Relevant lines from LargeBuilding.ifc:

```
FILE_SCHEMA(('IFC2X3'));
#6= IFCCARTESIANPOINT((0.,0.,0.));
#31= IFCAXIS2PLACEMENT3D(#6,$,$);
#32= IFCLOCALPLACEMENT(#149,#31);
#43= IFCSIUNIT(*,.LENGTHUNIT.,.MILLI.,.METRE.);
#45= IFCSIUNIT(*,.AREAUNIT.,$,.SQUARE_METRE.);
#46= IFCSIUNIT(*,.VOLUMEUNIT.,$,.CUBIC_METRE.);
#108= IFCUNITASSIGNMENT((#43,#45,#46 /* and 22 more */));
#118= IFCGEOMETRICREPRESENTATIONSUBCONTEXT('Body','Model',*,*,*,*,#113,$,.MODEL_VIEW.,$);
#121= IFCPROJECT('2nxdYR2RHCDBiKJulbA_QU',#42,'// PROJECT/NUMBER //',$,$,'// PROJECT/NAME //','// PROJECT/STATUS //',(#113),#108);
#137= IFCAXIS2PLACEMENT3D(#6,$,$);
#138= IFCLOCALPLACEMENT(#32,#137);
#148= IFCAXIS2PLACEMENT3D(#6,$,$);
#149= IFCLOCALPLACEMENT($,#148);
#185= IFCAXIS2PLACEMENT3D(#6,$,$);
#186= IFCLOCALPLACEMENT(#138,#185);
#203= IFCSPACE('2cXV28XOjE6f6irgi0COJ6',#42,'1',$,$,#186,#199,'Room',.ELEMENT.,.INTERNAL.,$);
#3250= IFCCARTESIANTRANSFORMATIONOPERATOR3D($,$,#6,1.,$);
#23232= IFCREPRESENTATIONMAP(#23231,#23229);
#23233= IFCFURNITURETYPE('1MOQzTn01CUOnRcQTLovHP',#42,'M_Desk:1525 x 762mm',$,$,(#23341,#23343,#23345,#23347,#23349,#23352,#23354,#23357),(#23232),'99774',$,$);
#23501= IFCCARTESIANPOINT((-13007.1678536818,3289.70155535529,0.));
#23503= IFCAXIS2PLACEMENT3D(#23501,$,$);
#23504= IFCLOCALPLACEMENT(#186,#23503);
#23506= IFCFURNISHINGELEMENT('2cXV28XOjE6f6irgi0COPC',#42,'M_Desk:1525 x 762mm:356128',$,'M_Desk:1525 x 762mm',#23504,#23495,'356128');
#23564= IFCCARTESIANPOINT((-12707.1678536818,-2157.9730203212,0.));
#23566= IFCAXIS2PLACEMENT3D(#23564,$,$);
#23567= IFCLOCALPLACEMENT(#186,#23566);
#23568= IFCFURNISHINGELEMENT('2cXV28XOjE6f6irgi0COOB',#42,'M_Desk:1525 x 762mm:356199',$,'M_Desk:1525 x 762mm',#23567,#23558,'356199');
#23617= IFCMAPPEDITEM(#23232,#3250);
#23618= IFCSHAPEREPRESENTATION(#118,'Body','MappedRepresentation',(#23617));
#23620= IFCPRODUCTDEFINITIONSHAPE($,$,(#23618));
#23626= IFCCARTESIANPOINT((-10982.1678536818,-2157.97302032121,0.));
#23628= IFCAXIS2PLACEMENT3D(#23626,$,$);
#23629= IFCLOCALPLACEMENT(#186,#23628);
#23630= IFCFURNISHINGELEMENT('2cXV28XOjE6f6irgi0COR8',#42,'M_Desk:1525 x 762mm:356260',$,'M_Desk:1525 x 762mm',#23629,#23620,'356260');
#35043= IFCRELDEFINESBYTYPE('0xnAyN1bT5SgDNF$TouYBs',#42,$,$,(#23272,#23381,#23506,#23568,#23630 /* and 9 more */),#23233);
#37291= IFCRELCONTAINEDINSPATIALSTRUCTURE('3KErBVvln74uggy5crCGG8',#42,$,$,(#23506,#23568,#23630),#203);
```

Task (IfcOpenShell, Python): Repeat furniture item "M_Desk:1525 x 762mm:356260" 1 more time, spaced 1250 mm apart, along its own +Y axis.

```python
import ifcopenshell
import ifcopenshell.api.geometry
import ifcopenshell.api.root
import ifcopenshell.util.element
import ifcopenshell.util.placement

model = ifcopenshell.open("LargeBuilding.ifc")


def reuse_history(source, copy):
    """copy_class also copies each property set's owner history, people and application; keep the originals."""
    for rel in copy.IsDefinedBy:
        if rel.is_a("IfcRelDefinesByProperties") and (history := rel.RelatingPropertyDefinition.OwnerHistory):
            rel.RelatingPropertyDefinition.OwnerHistory = source.OwnerHistory
            ifcopenshell.util.element.remove_deep2(model, history)


source = model.by_id(23630)
base = ifcopenshell.util.placement.get_local_placement(source.ObjectPlacement)
step = base[:3, 1] * 1250.0

for i in range(1, 2):
    copy = ifcopenshell.api.root.copy_class(model, product=source)
    copy.Representation = ifcopenshell.util.element.copy_deep(
        model, source.Representation, exclude=["IfcGeometricRepresentationContext", "IfcRepresentationMap"]
    )
    copy.Name = "M_Desk:1525 x 762mm"
    copy.Tag = None
    reuse_history(source, copy)
    matrix = base.copy()
    matrix[:3, 3] += i * step
    print("added at", matrix[:3, 3].round(3) + 0.0)
    ifcopenshell.api.geometry.edit_object_placement(model, product=copy, matrix=matrix, is_si=False)

model.write("LargeBuilding_edited.ifc")
```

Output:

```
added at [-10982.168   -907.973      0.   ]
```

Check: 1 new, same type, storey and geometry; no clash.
